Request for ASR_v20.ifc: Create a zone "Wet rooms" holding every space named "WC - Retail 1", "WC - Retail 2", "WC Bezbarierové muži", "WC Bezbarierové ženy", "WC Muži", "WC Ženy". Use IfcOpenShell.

First a look at what the model holds.

```python
import ifcopenshell

model = ifcopenshell.open("ASR_v20.ifc")
print(model.schema)
seen = {}
for space in model.by_type("IfcSpace"):
    seen[space.LongName] = seen.get(space.LongName, 0) + 1
for name, count in sorted(seen.items(), key=str):
    print(count, "x", name)
print("zones:", [z.Name for z in model.by_type("IfcZone")][:20])
```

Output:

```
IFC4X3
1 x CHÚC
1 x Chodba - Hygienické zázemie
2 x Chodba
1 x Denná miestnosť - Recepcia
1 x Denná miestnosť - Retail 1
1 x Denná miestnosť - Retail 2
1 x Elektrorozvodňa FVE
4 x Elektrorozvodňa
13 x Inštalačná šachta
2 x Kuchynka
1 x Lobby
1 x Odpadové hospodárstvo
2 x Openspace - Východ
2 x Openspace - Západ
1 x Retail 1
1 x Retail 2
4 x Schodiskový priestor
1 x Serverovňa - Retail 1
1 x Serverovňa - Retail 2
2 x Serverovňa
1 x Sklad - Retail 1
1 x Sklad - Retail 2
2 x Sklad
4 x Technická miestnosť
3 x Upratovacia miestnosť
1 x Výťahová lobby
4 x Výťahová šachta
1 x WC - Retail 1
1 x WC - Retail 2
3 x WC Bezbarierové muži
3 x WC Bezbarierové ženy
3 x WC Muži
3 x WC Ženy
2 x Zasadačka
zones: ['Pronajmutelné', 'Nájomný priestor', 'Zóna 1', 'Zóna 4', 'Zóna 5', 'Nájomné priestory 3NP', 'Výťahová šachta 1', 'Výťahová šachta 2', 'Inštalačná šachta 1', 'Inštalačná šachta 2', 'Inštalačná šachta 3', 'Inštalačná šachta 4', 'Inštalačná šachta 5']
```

```python
import ifcopenshell
import ifcopenshell.api.group
import ifcopenshell.api.root

model = ifcopenshell.open("ASR_v20.ifc")

names = {"WC - Retail 1", "WC - Retail 2", "WC Bezbarierové muži", "WC Bezbarierové ženy", "WC Muži", "WC Ženy"}
spaces = [s for s in model.by_type("IfcSpace") if s.LongName in names]

zone = ifcopenshell.api.root.create_entity(model, ifc_class="IfcZone", name="Wet rooms")
ifcopenshell.api.group.assign_group(model, products=spaces, group=zone)
print(len(spaces), "spaces in", zone.Name)

model.write("ASR_v20_updated.ifc")
```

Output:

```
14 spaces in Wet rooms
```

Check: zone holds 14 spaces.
